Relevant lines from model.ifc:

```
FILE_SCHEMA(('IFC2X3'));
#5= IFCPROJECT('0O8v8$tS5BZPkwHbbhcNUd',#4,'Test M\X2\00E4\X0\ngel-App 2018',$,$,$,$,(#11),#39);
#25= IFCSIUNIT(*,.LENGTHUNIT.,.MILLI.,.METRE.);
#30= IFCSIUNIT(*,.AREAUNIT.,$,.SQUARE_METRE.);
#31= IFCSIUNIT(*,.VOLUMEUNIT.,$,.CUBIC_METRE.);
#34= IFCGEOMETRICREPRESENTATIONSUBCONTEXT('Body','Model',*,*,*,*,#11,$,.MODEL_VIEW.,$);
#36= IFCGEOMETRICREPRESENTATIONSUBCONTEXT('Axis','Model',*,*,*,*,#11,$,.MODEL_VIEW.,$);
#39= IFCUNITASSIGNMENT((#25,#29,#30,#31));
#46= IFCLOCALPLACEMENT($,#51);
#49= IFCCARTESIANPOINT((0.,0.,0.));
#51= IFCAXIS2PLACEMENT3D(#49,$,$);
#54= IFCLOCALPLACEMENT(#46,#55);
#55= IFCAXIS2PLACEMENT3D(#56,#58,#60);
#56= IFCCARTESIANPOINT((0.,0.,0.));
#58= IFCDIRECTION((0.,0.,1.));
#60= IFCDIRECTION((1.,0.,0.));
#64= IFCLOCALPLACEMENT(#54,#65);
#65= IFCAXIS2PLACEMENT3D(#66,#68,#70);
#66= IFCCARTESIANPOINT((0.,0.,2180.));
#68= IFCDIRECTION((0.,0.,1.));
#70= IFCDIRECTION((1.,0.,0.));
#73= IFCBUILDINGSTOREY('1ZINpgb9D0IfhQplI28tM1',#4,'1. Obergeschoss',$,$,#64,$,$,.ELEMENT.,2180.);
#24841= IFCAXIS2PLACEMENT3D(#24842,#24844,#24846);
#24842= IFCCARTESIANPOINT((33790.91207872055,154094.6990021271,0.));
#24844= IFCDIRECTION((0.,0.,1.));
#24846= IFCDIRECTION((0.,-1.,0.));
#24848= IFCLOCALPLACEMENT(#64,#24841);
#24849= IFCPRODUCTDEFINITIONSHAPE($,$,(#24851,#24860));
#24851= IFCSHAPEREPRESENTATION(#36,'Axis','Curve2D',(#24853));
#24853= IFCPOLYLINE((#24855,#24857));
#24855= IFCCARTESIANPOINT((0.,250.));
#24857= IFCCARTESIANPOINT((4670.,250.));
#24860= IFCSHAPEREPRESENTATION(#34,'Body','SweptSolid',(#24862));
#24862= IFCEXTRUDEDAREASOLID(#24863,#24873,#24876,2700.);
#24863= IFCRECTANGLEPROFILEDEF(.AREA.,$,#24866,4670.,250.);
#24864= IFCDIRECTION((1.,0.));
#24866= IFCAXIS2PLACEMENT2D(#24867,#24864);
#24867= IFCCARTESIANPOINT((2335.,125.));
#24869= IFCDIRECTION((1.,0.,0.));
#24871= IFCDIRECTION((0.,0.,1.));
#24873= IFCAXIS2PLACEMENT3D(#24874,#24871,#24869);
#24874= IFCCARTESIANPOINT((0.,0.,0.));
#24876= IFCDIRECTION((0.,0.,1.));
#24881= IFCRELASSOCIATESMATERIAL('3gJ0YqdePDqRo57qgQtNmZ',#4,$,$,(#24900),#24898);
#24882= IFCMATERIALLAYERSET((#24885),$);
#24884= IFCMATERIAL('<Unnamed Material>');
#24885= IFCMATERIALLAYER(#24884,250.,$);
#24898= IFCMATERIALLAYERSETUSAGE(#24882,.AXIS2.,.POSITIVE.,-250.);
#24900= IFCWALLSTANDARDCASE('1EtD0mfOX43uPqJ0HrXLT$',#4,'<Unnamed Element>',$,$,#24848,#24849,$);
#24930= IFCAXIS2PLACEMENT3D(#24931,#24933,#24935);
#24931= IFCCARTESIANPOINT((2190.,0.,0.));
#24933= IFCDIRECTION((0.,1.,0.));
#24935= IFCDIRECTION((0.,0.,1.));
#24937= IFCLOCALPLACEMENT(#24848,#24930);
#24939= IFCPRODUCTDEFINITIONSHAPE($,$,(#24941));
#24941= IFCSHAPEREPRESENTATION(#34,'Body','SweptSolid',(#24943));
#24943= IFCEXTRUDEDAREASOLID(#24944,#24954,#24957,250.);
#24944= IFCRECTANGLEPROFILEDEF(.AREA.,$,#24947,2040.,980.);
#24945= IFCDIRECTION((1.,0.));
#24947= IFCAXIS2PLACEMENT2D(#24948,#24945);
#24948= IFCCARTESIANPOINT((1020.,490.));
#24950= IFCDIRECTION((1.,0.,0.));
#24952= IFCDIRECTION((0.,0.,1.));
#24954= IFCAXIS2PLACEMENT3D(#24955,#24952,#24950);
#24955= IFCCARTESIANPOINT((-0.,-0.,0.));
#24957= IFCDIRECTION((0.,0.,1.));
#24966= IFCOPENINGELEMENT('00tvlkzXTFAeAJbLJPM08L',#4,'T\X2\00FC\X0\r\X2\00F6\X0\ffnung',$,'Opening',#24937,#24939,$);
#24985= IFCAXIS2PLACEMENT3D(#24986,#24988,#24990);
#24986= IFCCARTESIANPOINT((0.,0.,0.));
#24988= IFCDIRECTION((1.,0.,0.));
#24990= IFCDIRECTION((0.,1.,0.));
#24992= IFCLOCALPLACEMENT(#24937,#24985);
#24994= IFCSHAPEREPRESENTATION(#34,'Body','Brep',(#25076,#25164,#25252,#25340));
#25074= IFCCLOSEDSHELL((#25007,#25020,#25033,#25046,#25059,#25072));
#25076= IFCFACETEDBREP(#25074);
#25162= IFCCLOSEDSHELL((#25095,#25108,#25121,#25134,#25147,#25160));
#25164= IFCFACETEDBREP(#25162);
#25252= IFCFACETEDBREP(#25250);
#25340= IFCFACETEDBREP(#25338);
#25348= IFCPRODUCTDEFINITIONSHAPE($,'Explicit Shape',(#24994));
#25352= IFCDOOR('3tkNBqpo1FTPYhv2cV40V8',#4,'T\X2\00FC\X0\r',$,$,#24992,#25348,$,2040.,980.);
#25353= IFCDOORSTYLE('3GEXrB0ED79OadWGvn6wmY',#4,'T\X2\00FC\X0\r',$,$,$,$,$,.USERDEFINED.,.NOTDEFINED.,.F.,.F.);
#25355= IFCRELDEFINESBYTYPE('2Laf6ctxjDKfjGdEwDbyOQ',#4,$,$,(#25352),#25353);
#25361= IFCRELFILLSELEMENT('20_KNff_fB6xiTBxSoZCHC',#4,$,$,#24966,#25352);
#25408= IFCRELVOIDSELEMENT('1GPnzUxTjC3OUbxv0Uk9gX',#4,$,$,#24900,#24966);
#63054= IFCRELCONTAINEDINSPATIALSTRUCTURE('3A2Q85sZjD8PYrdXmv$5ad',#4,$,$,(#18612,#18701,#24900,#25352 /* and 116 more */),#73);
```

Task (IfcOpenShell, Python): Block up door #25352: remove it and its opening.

```python
import ifcopenshell
import ifcopenshell.api.feature
import ifcopenshell.api.root
import ifcopenshell.geom
import ifcopenshell.util.shape

model = ifcopenshell.open("model.ifc")
settings = ifcopenshell.geom.settings()


def volume(element):
    """Net volume in cubic metres, openings subtracted."""
    shape = ifcopenshell.geom.create_shape(settings, element)
    return ifcopenshell.util.shape.get_volume(shape.geometry)


door = model.by_guid("3tkNBqpo1FTPYhv2cV40V8")
opening = door.FillsVoids[0].RelatingOpeningElement
wall = opening.VoidsElements[0].RelatingBuildingElement
before = volume(wall)

ifcopenshell.api.root.remove_product(model, product=door)
ifcopenshell.api.feature.remove_feature(model, feature=opening)

after = volume(wall)

print(f"wall volume {before:.3f} -> {after:.3f} m3")

model.write("model_rev.ifc")
```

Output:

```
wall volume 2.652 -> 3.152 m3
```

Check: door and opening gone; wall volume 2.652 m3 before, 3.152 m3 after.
